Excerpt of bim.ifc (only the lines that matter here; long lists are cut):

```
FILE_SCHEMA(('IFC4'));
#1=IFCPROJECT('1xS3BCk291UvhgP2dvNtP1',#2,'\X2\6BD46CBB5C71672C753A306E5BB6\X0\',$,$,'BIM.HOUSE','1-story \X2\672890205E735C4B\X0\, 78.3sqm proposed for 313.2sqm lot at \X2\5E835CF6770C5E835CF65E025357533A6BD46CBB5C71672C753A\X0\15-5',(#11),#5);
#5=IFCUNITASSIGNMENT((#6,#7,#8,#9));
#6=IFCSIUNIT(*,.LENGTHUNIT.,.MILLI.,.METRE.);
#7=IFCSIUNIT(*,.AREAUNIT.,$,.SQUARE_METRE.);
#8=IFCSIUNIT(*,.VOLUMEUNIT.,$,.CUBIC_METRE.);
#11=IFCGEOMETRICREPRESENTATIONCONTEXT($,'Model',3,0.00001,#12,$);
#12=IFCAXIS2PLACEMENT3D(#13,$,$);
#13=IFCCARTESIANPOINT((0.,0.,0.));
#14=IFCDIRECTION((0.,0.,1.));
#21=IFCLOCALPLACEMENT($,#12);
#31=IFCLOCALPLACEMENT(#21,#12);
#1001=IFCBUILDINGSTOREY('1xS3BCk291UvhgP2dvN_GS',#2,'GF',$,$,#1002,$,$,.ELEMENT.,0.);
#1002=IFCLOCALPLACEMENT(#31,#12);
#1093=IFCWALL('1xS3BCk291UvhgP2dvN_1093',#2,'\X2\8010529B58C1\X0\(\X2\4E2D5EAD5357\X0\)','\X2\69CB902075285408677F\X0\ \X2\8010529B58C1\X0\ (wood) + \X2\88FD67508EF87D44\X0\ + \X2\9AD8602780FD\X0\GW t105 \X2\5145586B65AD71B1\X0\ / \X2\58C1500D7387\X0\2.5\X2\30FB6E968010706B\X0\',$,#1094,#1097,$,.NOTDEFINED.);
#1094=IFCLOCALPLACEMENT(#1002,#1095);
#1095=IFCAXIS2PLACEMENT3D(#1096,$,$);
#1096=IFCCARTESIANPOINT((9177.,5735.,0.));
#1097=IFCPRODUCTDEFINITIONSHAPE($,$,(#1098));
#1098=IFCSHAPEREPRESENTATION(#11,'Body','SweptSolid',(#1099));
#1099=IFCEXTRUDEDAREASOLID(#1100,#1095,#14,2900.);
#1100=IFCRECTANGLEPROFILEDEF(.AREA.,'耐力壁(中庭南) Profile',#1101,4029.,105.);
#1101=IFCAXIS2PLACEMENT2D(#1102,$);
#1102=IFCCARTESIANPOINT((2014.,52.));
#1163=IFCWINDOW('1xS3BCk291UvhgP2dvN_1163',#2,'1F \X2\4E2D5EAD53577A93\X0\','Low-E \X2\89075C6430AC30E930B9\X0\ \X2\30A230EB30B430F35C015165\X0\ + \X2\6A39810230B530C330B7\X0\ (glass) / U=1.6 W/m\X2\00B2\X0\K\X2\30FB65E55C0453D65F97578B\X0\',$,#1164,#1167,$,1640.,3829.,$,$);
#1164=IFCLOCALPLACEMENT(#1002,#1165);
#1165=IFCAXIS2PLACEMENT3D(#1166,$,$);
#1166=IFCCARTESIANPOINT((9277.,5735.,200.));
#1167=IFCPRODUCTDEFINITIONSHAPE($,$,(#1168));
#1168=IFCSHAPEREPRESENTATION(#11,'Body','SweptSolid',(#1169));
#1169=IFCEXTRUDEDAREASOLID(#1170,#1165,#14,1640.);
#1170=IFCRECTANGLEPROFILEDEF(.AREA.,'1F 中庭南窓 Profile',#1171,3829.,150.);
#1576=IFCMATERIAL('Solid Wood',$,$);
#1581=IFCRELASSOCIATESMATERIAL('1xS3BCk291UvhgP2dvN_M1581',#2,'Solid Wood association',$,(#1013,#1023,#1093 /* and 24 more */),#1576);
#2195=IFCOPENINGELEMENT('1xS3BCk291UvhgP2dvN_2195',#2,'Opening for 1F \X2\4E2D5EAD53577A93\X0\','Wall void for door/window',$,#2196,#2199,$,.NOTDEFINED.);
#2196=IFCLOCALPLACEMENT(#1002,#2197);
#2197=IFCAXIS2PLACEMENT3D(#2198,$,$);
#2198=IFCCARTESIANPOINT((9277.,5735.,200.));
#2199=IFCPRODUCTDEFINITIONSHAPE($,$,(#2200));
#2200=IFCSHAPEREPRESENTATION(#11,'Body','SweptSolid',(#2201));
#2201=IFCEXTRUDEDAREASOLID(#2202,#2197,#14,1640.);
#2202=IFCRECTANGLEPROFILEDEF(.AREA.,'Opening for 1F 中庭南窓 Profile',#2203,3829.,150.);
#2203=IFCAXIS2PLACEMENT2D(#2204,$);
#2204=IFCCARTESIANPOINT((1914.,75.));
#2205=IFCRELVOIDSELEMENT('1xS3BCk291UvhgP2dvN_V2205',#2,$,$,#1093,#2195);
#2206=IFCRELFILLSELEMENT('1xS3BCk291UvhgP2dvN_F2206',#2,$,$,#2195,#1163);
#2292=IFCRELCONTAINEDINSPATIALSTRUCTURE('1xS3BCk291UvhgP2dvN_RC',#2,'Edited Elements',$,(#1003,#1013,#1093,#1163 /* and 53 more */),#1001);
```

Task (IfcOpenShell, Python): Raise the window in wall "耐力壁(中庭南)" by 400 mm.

```python
import numpy as np
import ifcopenshell
import ifcopenshell.api.geometry
import ifcopenshell.util.placement
import ifcopenshell.util.unit

model = ifcopenshell.open("bim.ifc")
unit_scale = ifcopenshell.util.unit.calculate_unit_scale(model)

window = model.by_id(1163)
opening = window.FillsVoids[0].RelatingOpeningElement
dz = 400.0

shift = np.array([0.0, 0.0, dz])
# The window is not placed relative to its opening, so move both.
for product in (opening, window):
    matrix = ifcopenshell.util.placement.get_local_placement(product.ObjectPlacement)
    matrix[:3, 3] += shift
    ifcopenshell.api.geometry.edit_object_placement(model, product=product, matrix=matrix, is_si=False)

print(f"moved by {dz * unit_scale:+.3f} m")

model.write("bim_updated.ifc")
```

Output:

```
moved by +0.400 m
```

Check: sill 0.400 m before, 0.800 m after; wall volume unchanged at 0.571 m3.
